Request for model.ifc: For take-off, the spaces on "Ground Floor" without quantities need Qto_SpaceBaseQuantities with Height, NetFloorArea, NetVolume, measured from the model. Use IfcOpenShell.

First a look at what the model holds.

```python
import ifcopenshell
import ifcopenshell.util.element
import ifcopenshell.util.unit

model = ifcopenshell.open("model.ifc")
print(model.schema)
for unit_type in ("LENGTHUNIT", "AREAUNIT", "VOLUMEUNIT"):
    print(unit_type, ifcopenshell.util.unit.calculate_unit_scale(model, unit_type))
storey = next(s for s in model.by_type("IfcBuildingStorey") if s.Name == "Ground Floor")
spaces = [e for e in ifcopenshell.util.element.get_decomposition(storey) if e.is_a("IfcSpace")]
for e in sorted(spaces, key=lambda e: e.id()):
    print(e.id(), e.is_a(), e.Name, list(ifcopenshell.util.element.get_psets(e, qtos_only=True)), sep=" | ")
```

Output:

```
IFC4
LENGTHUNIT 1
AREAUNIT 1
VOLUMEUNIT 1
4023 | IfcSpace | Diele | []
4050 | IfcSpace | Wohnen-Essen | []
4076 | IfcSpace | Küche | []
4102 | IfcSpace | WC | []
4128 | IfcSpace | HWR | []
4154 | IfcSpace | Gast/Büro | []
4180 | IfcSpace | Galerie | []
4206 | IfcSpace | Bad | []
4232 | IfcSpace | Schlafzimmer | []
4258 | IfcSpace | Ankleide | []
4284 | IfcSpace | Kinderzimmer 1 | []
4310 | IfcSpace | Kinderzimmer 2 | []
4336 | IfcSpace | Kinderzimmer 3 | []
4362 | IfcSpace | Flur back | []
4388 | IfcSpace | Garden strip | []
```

```python
import ifcopenshell
import ifcopenshell.api.pset
import ifcopenshell.geom
import ifcopenshell.util.element
import ifcopenshell.util.shape
import ifcopenshell.util.unit

model = ifcopenshell.open("model.ifc")
unit_scale = ifcopenshell.util.unit.calculate_unit_scale(model)
area_scale = ifcopenshell.util.unit.calculate_unit_scale(model, "AREAUNIT")
volume_scale = ifcopenshell.util.unit.calculate_unit_scale(model, "VOLUMEUNIT")
settings = ifcopenshell.geom.settings()

storey = next(s for s in model.by_type("IfcBuildingStorey") if s.Name == "Ground Floor")
spaces = [e for e in ifcopenshell.util.element.get_decomposition(storey) if e.is_a("IfcSpace")]

for e in sorted(spaces, key=lambda e: e.id()):
    if ifcopenshell.util.element.get_psets(e, qtos_only=True, should_inherit=False):
        continue
    # Geometry comes back in metres, in the element's own axes.
    shape = ifcopenshell.geom.create_shape(settings, e)
    values = {
        "Height": ifcopenshell.util.shape.get_z(shape.geometry) / unit_scale,
        "NetFloorArea": ifcopenshell.util.shape.get_footprint_area(shape.geometry) / area_scale,
        "NetVolume": ifcopenshell.util.shape.get_volume(shape.geometry) / volume_scale,
    }
    qto = ifcopenshell.api.pset.add_qto(model, product=e, name="Qto_SpaceBaseQuantities")
    ifcopenshell.api.pset.edit_qto(model, qto=qto, properties=values)
    print(e.id(), {k: round(v, 3) for k, v in values.items()})

model.write("model_rev.ifc")
```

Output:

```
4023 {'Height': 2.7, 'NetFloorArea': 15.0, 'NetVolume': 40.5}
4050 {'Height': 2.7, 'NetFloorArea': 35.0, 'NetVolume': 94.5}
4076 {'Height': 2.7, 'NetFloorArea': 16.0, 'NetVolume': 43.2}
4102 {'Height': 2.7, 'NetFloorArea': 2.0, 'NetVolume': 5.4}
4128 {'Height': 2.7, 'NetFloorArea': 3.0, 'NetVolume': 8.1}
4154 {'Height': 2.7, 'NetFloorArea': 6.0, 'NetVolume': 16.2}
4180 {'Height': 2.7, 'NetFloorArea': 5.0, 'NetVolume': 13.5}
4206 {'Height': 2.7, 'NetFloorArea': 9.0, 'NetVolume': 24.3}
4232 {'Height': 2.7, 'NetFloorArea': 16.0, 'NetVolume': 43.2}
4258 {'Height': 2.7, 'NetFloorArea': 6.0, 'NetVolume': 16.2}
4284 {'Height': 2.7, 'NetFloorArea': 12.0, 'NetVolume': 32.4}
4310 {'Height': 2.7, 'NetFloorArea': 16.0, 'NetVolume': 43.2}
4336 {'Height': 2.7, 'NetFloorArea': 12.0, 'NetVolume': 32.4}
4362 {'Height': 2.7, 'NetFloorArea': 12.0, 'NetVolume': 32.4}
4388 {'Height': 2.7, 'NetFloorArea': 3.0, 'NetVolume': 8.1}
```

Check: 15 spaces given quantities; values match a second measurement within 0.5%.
